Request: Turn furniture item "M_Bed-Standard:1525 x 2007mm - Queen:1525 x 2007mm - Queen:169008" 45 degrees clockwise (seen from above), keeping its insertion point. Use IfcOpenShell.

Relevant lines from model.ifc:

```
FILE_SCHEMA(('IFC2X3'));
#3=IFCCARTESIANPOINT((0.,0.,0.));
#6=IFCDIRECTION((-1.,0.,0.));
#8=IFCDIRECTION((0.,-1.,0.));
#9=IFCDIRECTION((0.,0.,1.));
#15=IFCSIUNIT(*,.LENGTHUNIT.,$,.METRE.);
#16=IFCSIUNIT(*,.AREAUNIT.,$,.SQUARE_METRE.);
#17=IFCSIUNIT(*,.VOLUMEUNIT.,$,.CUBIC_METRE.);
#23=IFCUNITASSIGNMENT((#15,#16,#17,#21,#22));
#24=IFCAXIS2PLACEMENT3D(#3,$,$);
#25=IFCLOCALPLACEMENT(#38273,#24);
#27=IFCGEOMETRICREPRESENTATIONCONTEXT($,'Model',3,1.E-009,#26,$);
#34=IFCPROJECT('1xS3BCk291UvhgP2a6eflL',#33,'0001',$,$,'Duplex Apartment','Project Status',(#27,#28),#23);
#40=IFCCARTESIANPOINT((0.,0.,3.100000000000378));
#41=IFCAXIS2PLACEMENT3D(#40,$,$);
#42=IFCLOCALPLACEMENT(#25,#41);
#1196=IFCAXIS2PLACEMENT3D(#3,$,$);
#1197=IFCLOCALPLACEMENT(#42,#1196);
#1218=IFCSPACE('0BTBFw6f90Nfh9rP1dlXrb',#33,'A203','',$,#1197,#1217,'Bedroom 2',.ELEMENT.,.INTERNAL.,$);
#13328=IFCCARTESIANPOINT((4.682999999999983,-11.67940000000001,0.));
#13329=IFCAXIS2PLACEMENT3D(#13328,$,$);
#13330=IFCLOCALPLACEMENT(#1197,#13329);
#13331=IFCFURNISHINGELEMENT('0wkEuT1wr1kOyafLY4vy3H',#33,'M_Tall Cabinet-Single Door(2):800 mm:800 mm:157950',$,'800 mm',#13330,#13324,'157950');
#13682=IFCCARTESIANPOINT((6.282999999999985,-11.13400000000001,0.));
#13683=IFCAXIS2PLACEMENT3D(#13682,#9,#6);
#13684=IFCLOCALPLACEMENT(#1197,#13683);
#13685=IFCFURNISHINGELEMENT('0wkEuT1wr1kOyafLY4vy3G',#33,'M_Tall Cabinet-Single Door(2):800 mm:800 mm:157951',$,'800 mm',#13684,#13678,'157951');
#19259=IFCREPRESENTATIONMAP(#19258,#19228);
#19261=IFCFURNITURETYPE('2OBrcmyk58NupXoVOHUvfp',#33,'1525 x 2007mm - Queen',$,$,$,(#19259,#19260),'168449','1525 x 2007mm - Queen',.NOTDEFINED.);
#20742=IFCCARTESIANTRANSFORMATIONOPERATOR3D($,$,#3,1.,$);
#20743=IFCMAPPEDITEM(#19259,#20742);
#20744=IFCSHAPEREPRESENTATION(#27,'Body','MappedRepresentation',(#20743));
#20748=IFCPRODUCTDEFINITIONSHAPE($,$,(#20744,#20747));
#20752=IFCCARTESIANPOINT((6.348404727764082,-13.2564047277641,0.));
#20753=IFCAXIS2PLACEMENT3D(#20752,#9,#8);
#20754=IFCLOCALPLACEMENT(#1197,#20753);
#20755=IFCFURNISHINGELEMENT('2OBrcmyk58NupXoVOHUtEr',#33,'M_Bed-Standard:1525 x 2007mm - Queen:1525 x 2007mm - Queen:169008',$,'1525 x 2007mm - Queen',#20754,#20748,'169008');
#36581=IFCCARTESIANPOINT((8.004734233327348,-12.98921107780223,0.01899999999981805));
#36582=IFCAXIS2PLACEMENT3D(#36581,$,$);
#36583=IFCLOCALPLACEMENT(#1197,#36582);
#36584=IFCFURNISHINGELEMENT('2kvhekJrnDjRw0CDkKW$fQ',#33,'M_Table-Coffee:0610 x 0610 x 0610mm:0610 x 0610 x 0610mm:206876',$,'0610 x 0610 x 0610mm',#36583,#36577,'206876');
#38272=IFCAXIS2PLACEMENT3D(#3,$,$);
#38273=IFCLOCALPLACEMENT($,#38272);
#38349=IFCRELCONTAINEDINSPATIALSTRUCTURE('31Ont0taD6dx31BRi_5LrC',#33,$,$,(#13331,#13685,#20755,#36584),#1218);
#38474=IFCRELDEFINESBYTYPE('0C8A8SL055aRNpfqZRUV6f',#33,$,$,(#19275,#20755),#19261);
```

```python
import ifcopenshell
import ifcopenshell.api.geometry
import ifcopenshell.util.placement

model = ifcopenshell.open("model.ifc")

item = model.by_id(20755)
matrix = ifcopenshell.util.placement.get_local_placement(item.ObjectPlacement)
matrix = matrix @ ifcopenshell.util.placement.rotation(-45, "Z")
ifcopenshell.api.geometry.edit_object_placement(model, product=item, matrix=matrix, is_si=False)

print(ifcopenshell.util.placement.get_local_placement(item.ObjectPlacement).round(3) + 0.0)

model.write("model-out.ifc")
```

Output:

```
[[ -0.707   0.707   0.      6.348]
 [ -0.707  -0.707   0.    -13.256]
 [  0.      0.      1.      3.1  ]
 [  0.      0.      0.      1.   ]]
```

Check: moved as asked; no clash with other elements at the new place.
